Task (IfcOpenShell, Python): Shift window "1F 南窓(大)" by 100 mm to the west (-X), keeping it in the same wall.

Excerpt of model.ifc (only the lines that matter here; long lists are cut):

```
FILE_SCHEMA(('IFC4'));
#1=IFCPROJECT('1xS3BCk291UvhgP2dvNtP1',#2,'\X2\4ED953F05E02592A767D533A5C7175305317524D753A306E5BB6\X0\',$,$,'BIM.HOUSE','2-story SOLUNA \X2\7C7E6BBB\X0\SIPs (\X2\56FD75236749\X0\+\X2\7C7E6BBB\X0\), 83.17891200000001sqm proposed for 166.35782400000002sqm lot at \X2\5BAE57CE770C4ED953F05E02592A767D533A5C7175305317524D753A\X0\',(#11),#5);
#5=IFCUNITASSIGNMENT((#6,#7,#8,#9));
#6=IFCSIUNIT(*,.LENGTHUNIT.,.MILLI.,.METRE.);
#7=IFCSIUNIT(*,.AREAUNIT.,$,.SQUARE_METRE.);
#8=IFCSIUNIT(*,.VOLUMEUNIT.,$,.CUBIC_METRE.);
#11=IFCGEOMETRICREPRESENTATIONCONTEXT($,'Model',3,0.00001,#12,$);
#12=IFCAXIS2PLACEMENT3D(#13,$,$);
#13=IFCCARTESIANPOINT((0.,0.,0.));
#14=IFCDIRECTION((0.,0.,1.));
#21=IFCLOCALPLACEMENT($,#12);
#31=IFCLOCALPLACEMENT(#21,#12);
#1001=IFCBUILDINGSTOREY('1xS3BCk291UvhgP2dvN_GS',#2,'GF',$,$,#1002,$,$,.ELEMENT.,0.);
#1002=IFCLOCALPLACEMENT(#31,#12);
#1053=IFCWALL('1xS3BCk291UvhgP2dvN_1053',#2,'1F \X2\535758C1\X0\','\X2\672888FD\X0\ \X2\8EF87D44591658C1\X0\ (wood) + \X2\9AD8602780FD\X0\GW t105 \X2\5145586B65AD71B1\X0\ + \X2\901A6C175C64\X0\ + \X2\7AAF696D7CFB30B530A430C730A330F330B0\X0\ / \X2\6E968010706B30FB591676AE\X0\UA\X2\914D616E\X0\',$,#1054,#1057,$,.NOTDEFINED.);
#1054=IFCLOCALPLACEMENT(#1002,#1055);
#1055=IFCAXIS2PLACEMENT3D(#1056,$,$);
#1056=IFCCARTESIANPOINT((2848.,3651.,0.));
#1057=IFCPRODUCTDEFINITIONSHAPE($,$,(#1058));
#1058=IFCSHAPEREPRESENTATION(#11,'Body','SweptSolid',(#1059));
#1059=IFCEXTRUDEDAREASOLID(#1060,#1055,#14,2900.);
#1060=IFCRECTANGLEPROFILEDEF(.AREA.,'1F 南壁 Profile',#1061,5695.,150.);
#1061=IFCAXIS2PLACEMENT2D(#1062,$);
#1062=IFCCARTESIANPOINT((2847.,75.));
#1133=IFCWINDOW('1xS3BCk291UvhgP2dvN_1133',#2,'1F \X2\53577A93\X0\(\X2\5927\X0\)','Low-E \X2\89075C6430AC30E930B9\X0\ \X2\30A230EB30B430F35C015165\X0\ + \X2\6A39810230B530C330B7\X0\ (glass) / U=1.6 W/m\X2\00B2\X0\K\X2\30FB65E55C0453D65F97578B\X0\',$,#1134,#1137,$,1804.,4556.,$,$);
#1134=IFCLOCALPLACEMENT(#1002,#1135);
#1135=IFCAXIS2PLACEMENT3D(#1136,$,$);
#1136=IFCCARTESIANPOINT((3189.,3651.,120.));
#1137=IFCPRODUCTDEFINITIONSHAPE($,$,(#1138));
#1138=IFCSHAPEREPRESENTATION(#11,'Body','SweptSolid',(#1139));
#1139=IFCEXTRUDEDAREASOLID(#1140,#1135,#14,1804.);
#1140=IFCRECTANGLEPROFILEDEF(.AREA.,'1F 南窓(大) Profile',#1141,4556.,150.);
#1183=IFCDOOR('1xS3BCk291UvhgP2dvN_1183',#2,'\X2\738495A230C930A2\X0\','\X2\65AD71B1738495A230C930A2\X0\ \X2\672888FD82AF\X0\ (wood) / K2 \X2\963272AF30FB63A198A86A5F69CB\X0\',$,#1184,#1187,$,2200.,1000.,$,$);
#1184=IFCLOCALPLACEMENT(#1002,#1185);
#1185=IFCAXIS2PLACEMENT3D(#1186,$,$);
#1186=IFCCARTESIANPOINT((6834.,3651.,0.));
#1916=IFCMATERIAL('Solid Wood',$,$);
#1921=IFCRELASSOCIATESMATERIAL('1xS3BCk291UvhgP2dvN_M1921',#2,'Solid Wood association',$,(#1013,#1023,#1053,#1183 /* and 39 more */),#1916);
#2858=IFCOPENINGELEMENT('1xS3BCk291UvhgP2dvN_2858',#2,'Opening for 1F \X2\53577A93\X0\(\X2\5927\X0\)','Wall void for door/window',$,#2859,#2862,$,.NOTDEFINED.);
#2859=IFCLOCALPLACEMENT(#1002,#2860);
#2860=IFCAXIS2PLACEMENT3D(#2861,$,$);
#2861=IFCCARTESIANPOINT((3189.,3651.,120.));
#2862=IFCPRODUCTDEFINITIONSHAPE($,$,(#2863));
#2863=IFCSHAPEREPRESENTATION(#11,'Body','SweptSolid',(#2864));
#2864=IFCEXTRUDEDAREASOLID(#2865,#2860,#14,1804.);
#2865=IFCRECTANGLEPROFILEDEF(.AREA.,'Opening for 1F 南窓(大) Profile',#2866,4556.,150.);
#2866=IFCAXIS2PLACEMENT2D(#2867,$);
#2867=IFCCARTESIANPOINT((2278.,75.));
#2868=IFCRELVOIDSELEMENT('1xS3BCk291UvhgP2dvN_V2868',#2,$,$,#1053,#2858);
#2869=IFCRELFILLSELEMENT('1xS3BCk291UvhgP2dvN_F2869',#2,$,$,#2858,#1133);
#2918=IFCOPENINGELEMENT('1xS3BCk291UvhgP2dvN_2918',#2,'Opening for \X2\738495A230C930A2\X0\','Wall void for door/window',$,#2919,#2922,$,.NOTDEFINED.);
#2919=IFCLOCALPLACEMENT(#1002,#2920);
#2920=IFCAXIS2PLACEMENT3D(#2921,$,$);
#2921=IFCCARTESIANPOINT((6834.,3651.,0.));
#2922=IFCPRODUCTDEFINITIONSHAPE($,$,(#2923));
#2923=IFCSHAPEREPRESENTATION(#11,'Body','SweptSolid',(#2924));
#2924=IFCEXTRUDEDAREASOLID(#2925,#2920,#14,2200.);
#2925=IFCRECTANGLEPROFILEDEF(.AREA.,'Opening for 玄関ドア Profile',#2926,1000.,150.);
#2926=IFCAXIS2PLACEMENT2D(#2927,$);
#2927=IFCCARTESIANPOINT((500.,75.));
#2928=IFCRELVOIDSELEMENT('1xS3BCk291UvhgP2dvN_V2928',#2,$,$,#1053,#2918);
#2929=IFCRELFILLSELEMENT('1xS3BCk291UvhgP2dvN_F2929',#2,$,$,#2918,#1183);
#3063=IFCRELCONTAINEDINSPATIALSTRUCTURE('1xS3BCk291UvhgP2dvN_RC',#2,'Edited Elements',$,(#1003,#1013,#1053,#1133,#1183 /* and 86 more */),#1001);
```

```python
import ifcopenshell
import ifcopenshell.api.geometry
import ifcopenshell.util.placement
import ifcopenshell.util.unit

model = ifcopenshell.open("model.ifc")
unit_scale = ifcopenshell.util.unit.calculate_unit_scale(model)

window = model.by_guid("1xS3BCk291UvhgP2dvN_1133")
opening = window.FillsVoids[0].RelatingOpeningElement
wall = opening.VoidsElements[0].RelatingBuildingElement

wall_matrix = ifcopenshell.util.placement.get_local_placement(wall.ObjectPlacement)
shift = wall_matrix[:3, 0] * -0.1 / unit_scale
before = ifcopenshell.util.placement.get_local_placement(window.ObjectPlacement)[:3, 3].copy()

# The window is not placed relative to its opening, so move both.
for product in (opening, window):
    matrix = ifcopenshell.util.placement.get_local_placement(product.ObjectPlacement)
    matrix[:3, 3] += shift
    ifcopenshell.api.geometry.edit_object_placement(model, product=product, matrix=matrix, is_si=False)

after = ifcopenshell.util.placement.get_local_placement(window.ObjectPlacement)[:3, 3]
print("window moved by", (after - before).round(3) + 0.0)

model.write("model_rev.ifc")
```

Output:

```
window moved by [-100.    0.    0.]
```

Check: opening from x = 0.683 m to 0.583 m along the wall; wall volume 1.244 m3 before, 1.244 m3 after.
